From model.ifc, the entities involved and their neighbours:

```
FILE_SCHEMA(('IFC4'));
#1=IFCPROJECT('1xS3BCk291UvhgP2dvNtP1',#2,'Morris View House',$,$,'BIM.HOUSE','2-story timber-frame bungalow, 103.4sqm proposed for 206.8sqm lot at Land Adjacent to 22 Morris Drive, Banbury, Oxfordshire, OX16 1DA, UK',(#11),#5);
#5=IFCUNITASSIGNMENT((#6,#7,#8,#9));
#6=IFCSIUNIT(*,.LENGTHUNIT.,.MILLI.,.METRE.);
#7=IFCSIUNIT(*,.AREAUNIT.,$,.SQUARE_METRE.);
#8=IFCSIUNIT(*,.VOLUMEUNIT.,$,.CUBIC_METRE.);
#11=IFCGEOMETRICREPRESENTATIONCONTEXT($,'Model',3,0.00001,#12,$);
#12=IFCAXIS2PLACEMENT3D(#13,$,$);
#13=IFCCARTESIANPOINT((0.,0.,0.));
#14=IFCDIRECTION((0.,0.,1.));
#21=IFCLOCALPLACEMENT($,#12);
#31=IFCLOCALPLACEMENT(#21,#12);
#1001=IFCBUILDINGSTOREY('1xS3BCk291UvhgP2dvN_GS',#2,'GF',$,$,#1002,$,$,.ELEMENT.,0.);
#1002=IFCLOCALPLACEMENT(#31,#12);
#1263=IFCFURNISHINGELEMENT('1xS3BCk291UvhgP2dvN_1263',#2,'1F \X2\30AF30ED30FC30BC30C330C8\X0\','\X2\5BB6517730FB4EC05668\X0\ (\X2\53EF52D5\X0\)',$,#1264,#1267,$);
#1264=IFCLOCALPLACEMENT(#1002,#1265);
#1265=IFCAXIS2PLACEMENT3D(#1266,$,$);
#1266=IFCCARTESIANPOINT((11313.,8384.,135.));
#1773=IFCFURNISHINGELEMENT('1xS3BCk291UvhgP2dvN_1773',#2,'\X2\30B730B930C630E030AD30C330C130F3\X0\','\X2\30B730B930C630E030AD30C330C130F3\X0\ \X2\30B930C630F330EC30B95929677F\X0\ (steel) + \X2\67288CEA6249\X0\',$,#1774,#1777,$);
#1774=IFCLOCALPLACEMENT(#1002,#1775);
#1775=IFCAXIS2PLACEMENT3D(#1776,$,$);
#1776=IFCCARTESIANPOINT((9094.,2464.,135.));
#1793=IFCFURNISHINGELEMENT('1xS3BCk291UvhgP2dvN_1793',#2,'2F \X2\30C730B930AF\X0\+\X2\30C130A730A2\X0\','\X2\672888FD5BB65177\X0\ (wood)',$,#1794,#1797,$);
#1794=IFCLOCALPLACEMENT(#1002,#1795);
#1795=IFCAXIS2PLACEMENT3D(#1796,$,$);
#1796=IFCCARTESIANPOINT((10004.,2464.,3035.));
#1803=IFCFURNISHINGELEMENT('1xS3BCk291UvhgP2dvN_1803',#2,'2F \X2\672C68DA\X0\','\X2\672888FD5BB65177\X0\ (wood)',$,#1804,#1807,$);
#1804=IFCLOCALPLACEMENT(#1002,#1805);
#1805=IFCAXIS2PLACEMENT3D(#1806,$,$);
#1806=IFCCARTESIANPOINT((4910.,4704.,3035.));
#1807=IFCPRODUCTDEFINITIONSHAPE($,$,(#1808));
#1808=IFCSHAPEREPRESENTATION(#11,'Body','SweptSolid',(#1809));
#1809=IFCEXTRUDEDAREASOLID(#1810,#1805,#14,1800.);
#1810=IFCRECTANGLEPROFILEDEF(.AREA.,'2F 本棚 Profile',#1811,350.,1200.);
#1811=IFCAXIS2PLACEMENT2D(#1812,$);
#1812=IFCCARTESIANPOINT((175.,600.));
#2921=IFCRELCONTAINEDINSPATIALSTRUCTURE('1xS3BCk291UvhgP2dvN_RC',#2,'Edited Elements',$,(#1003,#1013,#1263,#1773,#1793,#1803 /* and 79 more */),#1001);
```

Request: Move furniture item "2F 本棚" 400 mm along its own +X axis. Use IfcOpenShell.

```python
import ifcopenshell
import ifcopenshell.api.geometry
import ifcopenshell.util.placement

model = ifcopenshell.open("model.ifc")

item = model.by_id(1803)
matrix = ifcopenshell.util.placement.get_local_placement(item.ObjectPlacement)
matrix[:3, 3] += matrix[:3, 0] * 400.0
ifcopenshell.api.geometry.edit_object_placement(model, product=item, matrix=matrix, is_si=False)

print(ifcopenshell.util.placement.get_local_placement(item.ObjectPlacement).round(3) + 0.0)

model.write("model_edited.ifc")
```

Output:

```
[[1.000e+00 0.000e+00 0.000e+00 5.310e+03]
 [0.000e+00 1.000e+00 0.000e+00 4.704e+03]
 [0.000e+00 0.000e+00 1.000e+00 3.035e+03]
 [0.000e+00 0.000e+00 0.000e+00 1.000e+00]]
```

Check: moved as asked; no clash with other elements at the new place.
